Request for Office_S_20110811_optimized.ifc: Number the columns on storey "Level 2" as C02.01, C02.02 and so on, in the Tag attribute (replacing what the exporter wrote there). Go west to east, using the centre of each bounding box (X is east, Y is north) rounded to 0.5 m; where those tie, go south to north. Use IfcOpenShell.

First a look at what the model holds.

```python
import ifcopenshell
import ifcopenshell.util.element
import ifcopenshell.util.placement

model = ifcopenshell.open("Office_S_20110811_optimized.ifc")
print(model.schema)
storey = next(s for s in model.by_type("IfcBuildingStorey") if s.Name == "Level 2")
columns = [e for e in ifcopenshell.util.element.get_decomposition(storey) if e.is_a("IfcColumn")]
for e in sorted(columns, key=lambda e: e.id()):
    origin = ifcopenshell.util.placement.get_local_placement(e.ObjectPlacement)[:3, 3]
    print(e.id(), e.Tag, e.Name, origin.round(2) + 0.0, sep=" | ")
```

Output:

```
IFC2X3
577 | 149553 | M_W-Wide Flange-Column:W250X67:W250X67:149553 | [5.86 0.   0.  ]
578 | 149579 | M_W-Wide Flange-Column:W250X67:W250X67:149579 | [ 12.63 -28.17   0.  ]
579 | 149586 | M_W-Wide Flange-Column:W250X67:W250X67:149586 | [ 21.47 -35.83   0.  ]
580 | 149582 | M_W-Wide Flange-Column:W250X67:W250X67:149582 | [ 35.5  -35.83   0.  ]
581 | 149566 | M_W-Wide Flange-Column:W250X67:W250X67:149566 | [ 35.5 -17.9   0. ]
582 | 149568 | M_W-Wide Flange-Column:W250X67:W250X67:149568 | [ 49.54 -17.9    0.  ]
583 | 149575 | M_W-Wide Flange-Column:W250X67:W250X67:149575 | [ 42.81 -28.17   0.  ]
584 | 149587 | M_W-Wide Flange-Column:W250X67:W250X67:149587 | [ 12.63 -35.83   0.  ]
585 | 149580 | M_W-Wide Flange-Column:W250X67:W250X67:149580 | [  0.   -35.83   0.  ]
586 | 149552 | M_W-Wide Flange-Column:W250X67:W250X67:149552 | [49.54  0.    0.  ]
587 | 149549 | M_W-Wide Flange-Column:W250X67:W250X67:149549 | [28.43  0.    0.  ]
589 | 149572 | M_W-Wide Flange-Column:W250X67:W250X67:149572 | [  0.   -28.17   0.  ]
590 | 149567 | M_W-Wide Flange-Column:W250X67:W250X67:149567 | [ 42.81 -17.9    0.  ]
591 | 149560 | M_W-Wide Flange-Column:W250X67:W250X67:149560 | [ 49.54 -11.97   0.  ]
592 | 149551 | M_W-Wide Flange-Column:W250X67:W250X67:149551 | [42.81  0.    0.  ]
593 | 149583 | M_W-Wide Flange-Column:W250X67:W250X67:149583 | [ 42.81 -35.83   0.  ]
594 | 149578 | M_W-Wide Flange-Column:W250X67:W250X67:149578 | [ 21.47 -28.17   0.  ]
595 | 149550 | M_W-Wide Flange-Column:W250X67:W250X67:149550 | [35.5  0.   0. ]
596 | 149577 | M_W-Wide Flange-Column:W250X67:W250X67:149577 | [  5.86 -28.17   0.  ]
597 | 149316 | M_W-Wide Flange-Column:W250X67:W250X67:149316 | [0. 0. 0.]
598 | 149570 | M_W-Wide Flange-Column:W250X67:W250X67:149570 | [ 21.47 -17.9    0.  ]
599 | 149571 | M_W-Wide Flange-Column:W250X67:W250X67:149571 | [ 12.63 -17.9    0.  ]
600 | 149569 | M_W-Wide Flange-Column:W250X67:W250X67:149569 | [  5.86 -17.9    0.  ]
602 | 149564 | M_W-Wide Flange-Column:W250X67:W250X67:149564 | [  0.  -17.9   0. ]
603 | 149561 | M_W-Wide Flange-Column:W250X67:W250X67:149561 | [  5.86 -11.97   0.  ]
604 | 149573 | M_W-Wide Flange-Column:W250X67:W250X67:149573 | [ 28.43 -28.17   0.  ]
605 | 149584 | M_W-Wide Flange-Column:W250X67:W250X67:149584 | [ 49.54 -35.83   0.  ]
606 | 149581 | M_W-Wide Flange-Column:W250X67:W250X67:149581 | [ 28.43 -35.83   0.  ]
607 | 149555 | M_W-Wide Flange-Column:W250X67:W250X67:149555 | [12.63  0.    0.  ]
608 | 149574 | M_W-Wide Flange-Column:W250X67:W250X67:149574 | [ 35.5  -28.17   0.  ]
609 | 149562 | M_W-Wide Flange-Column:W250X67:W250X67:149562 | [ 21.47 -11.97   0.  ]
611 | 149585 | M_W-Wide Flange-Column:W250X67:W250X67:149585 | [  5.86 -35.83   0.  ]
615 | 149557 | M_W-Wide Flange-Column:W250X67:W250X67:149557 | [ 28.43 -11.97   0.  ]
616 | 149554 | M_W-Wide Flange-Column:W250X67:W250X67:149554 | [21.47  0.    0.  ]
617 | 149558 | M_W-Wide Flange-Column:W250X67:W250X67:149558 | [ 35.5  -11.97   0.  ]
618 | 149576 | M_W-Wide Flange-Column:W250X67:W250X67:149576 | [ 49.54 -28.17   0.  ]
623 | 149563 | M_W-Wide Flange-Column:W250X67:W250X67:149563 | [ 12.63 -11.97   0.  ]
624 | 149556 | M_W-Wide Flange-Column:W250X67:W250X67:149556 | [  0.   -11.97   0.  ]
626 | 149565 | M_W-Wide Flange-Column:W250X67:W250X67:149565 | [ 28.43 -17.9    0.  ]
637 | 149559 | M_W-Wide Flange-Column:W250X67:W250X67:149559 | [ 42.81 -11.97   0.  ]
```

```python
import ifcopenshell
import ifcopenshell.geom
import ifcopenshell.util.element
import ifcopenshell.util.shape

model = ifcopenshell.open("Office_S_20110811_optimized.ifc")
settings = ifcopenshell.geom.settings()
settings.set("use-world-coords", True)


def centre(element):
    shape = ifcopenshell.geom.create_shape(settings, element)
    return ifcopenshell.util.shape.get_bbox_centroid(shape.geometry)


storey = next(s for s in model.by_type("IfcBuildingStorey") if s.Name == "Level 2")
columns = [e for e in ifcopenshell.util.element.get_decomposition(storey) if e.is_a("IfcColumn")]

# Insertion points can sit at a corner or the storey origin, so sort by the geometry (in metres).
centres = {e: centre(e) for e in columns}
columns.sort(key=lambda e: (round(centres[e][0] / 0.5), centres[e][1]))

for i, e in enumerate(columns, start=1):
    number = f"C02.{i:02d}"
    e.Tag = number
    print(e.id(), number)

model.write("Office_S_20110811_optimized_rev.ifc")
```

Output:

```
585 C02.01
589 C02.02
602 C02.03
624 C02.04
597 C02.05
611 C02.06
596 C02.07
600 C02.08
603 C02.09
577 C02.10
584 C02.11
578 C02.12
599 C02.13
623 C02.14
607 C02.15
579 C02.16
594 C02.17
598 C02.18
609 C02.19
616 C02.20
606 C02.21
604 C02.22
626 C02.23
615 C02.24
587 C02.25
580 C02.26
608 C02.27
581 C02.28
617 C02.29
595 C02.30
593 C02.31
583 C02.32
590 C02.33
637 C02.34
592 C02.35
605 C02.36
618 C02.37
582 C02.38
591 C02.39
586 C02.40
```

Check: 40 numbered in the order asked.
